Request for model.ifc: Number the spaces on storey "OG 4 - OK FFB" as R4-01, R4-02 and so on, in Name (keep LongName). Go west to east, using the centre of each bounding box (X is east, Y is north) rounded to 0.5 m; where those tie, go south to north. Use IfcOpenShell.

First a look at what the model holds.

```python
import ifcopenshell
import ifcopenshell.util.element
import ifcopenshell.util.placement

model = ifcopenshell.open("model.ifc")
print(model.schema)
storey = next(s for s in model.by_type("IfcBuildingStorey") if s.Name == "OG 4 - OK FFB")
spaces = [e for e in ifcopenshell.util.element.get_decomposition(storey) if e.is_a("IfcSpace")]
for e in sorted(spaces, key=lambda e: e.id()):
    origin = ifcopenshell.util.placement.get_local_placement(e.ObjectPlacement)[:3, 3]
    print(e.id(), e.Name, e.LongName, origin.round(2) + 0.0, sep=" | ")
```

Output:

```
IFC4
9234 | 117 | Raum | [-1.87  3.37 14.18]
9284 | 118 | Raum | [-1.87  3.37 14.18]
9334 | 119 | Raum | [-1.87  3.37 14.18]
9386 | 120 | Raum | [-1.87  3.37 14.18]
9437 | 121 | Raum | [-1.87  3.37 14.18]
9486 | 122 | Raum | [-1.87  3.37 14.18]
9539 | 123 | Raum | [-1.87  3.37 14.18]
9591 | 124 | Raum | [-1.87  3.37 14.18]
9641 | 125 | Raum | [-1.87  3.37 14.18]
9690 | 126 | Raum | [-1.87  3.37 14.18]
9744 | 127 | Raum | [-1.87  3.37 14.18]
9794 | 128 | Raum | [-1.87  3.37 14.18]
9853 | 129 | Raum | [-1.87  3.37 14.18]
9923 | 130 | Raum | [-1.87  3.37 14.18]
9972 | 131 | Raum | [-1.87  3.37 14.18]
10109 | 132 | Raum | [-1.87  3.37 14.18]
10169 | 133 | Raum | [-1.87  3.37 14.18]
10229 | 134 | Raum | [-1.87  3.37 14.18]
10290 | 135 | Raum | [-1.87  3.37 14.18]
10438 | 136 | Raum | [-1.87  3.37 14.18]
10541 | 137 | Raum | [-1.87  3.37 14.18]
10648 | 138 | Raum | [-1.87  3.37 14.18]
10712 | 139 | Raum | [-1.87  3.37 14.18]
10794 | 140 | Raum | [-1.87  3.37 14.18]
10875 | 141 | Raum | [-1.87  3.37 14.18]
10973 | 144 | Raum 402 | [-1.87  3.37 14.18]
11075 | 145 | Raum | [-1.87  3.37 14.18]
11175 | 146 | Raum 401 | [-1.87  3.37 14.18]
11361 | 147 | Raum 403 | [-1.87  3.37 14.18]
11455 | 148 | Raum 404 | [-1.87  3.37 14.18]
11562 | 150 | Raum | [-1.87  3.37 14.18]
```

```python
import ifcopenshell
import ifcopenshell.geom
import ifcopenshell.util.element
import ifcopenshell.util.shape

model = ifcopenshell.open("model.ifc")
settings = ifcopenshell.geom.settings()
settings.set("use-world-coords", True)


def centre(element):
    shape = ifcopenshell.geom.create_shape(settings, element)
    return ifcopenshell.util.shape.get_bbox_centroid(shape.geometry)


storey = next(s for s in model.by_type("IfcBuildingStorey") if s.Name == "OG 4 - OK FFB")
spaces = [e for e in ifcopenshell.util.element.get_decomposition(storey) if e.is_a("IfcSpace")]

# Insertion points can sit at a corner or the storey origin, so sort by the geometry (in metres).
centres = {e: centre(e) for e in spaces}
spaces.sort(key=lambda e: (round(centres[e][0] / 0.5), centres[e][1]))

for i, e in enumerate(spaces, start=1):
    number = f"R4-{i:02d}"
    e.Name = number
    print(e.id(), number)

model.write("model_rev.ifc")
```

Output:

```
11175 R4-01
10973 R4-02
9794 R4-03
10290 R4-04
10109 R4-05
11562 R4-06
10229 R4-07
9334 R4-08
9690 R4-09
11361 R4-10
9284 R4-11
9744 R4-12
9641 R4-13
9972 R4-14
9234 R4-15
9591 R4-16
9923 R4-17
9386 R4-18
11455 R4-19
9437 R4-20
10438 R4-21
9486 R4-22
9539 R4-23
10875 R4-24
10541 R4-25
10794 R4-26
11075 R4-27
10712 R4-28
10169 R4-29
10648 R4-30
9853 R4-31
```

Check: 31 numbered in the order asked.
